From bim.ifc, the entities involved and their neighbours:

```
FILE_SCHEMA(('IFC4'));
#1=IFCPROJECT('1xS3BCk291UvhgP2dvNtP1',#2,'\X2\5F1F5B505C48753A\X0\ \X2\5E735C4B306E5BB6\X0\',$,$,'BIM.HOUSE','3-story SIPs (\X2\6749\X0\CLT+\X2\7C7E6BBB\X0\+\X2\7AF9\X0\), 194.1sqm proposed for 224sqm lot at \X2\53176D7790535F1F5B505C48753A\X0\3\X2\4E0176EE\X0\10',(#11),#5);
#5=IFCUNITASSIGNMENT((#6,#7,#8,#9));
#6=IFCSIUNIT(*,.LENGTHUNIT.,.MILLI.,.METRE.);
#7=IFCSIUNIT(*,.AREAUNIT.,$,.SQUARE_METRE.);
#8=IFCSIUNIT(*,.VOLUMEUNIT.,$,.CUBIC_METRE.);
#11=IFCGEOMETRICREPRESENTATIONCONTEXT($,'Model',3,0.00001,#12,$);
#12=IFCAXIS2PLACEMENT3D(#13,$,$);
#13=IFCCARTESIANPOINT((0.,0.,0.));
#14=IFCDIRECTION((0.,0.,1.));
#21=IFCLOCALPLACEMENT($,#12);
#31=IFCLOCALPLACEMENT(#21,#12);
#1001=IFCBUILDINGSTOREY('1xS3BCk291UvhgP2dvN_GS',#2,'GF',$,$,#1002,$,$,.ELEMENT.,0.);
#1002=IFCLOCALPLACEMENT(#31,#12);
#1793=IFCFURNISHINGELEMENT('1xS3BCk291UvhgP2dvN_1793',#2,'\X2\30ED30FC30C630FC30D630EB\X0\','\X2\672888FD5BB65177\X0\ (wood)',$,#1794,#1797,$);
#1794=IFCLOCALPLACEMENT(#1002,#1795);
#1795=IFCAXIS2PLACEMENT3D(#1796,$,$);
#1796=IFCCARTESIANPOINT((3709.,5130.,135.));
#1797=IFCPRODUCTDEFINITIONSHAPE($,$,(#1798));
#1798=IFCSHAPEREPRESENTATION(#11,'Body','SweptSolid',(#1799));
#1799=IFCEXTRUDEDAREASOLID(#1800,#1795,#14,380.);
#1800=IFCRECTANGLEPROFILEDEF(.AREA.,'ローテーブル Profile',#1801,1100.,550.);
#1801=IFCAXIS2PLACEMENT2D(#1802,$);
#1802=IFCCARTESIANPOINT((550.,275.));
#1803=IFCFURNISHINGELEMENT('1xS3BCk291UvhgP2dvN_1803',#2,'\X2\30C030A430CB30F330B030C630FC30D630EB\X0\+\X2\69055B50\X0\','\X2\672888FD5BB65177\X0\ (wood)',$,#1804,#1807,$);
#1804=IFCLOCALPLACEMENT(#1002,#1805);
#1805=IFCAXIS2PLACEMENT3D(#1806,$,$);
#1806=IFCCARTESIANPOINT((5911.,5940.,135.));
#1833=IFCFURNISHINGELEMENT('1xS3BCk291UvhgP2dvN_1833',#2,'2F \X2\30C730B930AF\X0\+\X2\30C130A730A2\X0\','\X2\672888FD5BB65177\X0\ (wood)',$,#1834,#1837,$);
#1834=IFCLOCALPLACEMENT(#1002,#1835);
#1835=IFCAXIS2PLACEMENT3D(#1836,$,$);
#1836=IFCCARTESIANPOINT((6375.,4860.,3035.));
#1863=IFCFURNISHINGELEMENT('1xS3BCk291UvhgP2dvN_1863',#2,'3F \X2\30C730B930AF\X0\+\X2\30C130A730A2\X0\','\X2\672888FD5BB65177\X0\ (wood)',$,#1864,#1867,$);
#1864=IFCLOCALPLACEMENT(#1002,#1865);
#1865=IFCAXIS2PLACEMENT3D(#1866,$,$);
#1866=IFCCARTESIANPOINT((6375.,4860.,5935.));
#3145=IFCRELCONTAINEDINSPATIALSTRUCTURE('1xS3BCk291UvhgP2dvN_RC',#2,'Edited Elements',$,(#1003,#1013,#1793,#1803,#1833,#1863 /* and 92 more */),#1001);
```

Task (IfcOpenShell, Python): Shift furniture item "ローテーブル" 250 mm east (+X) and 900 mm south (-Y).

```python
import ifcopenshell
import ifcopenshell.api.geometry
import ifcopenshell.util.placement
import ifcopenshell.util.unit

model = ifcopenshell.open("bim.ifc")
unit_scale = ifcopenshell.util.unit.calculate_unit_scale(model)

item = model.by_id(1793)
matrix = ifcopenshell.util.placement.get_local_placement(item.ObjectPlacement)
matrix[0, 3] += 0.25 / unit_scale
matrix[1, 3] -= 0.9 / unit_scale
ifcopenshell.api.geometry.edit_object_placement(model, product=item, matrix=matrix, is_si=False)

print(ifcopenshell.util.placement.get_local_placement(item.ObjectPlacement).round(3) + 0.0)

model.write("bim_edited.ifc")
```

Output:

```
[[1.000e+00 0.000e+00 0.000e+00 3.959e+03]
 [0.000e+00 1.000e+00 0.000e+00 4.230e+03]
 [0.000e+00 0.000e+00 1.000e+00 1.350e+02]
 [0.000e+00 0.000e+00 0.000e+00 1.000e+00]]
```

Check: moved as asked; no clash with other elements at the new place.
